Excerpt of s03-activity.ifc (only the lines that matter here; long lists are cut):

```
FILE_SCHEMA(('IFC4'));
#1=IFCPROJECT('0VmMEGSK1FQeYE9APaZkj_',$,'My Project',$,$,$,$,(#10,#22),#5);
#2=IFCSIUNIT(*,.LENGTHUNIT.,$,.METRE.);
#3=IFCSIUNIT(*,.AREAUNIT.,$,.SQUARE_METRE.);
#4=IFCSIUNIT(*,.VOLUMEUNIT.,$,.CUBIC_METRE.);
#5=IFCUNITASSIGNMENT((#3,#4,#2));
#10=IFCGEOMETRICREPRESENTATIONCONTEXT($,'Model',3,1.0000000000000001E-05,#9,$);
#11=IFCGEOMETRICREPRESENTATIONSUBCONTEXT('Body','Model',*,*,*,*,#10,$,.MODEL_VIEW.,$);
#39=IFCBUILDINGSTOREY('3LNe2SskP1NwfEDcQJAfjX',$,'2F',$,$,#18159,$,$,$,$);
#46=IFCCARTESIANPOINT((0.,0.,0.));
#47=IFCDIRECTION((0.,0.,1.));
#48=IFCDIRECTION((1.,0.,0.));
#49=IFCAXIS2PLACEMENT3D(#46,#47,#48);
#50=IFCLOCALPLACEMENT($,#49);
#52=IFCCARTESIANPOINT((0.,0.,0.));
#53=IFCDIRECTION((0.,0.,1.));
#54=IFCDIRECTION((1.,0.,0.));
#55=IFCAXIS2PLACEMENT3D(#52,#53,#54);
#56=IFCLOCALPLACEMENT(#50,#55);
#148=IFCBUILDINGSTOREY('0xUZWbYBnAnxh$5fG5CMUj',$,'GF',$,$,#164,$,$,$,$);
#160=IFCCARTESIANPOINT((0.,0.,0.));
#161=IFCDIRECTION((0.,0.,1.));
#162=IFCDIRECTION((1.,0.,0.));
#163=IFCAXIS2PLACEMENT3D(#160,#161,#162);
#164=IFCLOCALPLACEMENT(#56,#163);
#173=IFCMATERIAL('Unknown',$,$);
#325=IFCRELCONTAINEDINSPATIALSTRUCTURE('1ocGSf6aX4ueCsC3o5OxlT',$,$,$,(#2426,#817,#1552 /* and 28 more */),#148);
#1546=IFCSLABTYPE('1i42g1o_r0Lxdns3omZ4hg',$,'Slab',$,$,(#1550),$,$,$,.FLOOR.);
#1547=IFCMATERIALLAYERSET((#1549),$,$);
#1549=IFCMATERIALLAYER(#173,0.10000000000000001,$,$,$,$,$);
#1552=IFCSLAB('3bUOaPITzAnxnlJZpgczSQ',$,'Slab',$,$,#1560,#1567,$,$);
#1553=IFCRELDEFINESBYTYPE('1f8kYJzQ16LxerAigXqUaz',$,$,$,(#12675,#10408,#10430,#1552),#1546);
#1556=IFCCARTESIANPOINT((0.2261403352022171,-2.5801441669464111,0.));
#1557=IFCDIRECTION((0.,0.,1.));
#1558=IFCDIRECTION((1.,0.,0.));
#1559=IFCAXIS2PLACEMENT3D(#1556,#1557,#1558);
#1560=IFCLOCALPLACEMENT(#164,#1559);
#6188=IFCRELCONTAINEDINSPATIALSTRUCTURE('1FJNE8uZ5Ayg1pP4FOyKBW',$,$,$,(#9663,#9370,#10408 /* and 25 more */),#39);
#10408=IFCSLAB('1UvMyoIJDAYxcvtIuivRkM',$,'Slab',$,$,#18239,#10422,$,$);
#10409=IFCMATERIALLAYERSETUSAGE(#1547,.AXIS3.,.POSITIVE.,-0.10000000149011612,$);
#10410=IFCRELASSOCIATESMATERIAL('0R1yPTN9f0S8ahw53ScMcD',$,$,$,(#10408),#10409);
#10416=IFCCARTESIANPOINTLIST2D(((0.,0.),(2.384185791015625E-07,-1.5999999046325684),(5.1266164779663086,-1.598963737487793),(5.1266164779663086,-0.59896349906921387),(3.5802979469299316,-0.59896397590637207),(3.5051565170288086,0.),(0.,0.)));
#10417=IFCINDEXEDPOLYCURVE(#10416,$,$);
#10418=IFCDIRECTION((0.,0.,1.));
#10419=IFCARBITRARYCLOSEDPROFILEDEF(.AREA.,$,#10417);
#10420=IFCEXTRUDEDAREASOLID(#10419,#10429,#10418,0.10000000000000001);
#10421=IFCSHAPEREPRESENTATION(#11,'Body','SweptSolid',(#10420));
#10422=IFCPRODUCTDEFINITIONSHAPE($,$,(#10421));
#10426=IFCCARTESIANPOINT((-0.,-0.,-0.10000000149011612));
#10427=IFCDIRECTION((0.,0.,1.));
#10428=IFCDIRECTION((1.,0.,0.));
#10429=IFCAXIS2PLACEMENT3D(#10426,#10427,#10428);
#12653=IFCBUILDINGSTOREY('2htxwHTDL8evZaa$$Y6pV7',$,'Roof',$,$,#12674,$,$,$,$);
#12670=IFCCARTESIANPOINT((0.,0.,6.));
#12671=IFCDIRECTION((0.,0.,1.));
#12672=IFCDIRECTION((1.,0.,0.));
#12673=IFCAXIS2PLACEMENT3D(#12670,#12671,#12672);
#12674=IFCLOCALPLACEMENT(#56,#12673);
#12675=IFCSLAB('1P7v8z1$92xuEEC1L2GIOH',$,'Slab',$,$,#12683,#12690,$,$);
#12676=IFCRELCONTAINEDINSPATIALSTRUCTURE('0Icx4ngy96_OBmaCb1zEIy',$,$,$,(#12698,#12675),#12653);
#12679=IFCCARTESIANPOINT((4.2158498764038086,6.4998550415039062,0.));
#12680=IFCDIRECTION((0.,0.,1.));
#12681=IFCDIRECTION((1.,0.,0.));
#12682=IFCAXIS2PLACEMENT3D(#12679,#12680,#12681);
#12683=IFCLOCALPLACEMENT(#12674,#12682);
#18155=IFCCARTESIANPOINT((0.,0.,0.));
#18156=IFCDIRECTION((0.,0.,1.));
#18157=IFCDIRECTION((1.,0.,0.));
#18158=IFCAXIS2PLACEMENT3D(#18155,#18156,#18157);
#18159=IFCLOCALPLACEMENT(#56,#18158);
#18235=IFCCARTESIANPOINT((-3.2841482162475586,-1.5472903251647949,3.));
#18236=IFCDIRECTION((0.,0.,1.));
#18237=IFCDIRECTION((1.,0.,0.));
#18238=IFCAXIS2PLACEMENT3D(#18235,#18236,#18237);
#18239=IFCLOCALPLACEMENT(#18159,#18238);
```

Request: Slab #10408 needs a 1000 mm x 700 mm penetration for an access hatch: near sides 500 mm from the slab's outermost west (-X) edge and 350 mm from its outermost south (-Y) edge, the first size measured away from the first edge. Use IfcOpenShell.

```python
import numpy as np
import ifcopenshell
import ifcopenshell.api.feature
import ifcopenshell.api.geometry
import ifcopenshell.api.root
import ifcopenshell.geom
import ifcopenshell.util.placement
import ifcopenshell.util.representation
import ifcopenshell.util.shape
import ifcopenshell.util.unit

model = ifcopenshell.open("s03-activity.ifc")
unit_scale = ifcopenshell.util.unit.calculate_unit_scale(model)
settings = ifcopenshell.geom.settings()


def volume(element):
    """Net volume in cubic metres, openings subtracted."""
    shape = ifcopenshell.geom.create_shape(settings, element)
    return ifcopenshell.util.shape.get_volume(shape.geometry)


slab = model.by_guid("1UvMyoIJDAYxcvtIuivRkM")
before = volume(slab)

# Extent in the slab's own axes, in metres. The edges named are its -X and -Y sides.
slab_shape = ifcopenshell.geom.create_shape(settings, slab)
vertices = ifcopenshell.util.shape.get_vertices(slab_shape.geometry)
x_min, y_min, bottom = vertices.min(axis=0)
top = vertices[:, 2].max()

opening = ifcopenshell.api.root.create_entity(model, ifc_class="IfcOpeningElement", name="Access hatch opening", predefined_type="OPENING")
context = ifcopenshell.util.representation.get_context(model, "Model", "Body", "MODEL_VIEW")
width, depth = 1, 0.7
outline = [(0.0, 0.0), (width, 0.0), (width, depth), (0.0, depth), (0.0, 0.0)]
# Overshoot both faces by 50 mm so the cut is clean.
shape = ifcopenshell.api.geometry.add_slab_representation(
    model, context=context, depth=top - bottom + 0.1, polyline=outline
)
ifcopenshell.api.geometry.assign_representation(model, product=opening, representation=shape)

matrix = ifcopenshell.util.placement.get_local_placement(slab.ObjectPlacement)
matrix[:, 3] = matrix @ np.append(np.array([x_min + 0.5, y_min + 0.35, bottom - 0.05]) / unit_scale, 1.0)
ifcopenshell.api.geometry.edit_object_placement(model, product=opening, matrix=matrix, is_si=False)
ifcopenshell.api.feature.add_feature(model, feature=opening, element=slab)

after = volume(slab)

print(f"slab volume {before:.3f} -> {after:.3f} m3")

model.write("s03-activity_v2.ifc")
```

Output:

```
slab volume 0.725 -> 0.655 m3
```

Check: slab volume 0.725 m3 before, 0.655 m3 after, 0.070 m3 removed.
